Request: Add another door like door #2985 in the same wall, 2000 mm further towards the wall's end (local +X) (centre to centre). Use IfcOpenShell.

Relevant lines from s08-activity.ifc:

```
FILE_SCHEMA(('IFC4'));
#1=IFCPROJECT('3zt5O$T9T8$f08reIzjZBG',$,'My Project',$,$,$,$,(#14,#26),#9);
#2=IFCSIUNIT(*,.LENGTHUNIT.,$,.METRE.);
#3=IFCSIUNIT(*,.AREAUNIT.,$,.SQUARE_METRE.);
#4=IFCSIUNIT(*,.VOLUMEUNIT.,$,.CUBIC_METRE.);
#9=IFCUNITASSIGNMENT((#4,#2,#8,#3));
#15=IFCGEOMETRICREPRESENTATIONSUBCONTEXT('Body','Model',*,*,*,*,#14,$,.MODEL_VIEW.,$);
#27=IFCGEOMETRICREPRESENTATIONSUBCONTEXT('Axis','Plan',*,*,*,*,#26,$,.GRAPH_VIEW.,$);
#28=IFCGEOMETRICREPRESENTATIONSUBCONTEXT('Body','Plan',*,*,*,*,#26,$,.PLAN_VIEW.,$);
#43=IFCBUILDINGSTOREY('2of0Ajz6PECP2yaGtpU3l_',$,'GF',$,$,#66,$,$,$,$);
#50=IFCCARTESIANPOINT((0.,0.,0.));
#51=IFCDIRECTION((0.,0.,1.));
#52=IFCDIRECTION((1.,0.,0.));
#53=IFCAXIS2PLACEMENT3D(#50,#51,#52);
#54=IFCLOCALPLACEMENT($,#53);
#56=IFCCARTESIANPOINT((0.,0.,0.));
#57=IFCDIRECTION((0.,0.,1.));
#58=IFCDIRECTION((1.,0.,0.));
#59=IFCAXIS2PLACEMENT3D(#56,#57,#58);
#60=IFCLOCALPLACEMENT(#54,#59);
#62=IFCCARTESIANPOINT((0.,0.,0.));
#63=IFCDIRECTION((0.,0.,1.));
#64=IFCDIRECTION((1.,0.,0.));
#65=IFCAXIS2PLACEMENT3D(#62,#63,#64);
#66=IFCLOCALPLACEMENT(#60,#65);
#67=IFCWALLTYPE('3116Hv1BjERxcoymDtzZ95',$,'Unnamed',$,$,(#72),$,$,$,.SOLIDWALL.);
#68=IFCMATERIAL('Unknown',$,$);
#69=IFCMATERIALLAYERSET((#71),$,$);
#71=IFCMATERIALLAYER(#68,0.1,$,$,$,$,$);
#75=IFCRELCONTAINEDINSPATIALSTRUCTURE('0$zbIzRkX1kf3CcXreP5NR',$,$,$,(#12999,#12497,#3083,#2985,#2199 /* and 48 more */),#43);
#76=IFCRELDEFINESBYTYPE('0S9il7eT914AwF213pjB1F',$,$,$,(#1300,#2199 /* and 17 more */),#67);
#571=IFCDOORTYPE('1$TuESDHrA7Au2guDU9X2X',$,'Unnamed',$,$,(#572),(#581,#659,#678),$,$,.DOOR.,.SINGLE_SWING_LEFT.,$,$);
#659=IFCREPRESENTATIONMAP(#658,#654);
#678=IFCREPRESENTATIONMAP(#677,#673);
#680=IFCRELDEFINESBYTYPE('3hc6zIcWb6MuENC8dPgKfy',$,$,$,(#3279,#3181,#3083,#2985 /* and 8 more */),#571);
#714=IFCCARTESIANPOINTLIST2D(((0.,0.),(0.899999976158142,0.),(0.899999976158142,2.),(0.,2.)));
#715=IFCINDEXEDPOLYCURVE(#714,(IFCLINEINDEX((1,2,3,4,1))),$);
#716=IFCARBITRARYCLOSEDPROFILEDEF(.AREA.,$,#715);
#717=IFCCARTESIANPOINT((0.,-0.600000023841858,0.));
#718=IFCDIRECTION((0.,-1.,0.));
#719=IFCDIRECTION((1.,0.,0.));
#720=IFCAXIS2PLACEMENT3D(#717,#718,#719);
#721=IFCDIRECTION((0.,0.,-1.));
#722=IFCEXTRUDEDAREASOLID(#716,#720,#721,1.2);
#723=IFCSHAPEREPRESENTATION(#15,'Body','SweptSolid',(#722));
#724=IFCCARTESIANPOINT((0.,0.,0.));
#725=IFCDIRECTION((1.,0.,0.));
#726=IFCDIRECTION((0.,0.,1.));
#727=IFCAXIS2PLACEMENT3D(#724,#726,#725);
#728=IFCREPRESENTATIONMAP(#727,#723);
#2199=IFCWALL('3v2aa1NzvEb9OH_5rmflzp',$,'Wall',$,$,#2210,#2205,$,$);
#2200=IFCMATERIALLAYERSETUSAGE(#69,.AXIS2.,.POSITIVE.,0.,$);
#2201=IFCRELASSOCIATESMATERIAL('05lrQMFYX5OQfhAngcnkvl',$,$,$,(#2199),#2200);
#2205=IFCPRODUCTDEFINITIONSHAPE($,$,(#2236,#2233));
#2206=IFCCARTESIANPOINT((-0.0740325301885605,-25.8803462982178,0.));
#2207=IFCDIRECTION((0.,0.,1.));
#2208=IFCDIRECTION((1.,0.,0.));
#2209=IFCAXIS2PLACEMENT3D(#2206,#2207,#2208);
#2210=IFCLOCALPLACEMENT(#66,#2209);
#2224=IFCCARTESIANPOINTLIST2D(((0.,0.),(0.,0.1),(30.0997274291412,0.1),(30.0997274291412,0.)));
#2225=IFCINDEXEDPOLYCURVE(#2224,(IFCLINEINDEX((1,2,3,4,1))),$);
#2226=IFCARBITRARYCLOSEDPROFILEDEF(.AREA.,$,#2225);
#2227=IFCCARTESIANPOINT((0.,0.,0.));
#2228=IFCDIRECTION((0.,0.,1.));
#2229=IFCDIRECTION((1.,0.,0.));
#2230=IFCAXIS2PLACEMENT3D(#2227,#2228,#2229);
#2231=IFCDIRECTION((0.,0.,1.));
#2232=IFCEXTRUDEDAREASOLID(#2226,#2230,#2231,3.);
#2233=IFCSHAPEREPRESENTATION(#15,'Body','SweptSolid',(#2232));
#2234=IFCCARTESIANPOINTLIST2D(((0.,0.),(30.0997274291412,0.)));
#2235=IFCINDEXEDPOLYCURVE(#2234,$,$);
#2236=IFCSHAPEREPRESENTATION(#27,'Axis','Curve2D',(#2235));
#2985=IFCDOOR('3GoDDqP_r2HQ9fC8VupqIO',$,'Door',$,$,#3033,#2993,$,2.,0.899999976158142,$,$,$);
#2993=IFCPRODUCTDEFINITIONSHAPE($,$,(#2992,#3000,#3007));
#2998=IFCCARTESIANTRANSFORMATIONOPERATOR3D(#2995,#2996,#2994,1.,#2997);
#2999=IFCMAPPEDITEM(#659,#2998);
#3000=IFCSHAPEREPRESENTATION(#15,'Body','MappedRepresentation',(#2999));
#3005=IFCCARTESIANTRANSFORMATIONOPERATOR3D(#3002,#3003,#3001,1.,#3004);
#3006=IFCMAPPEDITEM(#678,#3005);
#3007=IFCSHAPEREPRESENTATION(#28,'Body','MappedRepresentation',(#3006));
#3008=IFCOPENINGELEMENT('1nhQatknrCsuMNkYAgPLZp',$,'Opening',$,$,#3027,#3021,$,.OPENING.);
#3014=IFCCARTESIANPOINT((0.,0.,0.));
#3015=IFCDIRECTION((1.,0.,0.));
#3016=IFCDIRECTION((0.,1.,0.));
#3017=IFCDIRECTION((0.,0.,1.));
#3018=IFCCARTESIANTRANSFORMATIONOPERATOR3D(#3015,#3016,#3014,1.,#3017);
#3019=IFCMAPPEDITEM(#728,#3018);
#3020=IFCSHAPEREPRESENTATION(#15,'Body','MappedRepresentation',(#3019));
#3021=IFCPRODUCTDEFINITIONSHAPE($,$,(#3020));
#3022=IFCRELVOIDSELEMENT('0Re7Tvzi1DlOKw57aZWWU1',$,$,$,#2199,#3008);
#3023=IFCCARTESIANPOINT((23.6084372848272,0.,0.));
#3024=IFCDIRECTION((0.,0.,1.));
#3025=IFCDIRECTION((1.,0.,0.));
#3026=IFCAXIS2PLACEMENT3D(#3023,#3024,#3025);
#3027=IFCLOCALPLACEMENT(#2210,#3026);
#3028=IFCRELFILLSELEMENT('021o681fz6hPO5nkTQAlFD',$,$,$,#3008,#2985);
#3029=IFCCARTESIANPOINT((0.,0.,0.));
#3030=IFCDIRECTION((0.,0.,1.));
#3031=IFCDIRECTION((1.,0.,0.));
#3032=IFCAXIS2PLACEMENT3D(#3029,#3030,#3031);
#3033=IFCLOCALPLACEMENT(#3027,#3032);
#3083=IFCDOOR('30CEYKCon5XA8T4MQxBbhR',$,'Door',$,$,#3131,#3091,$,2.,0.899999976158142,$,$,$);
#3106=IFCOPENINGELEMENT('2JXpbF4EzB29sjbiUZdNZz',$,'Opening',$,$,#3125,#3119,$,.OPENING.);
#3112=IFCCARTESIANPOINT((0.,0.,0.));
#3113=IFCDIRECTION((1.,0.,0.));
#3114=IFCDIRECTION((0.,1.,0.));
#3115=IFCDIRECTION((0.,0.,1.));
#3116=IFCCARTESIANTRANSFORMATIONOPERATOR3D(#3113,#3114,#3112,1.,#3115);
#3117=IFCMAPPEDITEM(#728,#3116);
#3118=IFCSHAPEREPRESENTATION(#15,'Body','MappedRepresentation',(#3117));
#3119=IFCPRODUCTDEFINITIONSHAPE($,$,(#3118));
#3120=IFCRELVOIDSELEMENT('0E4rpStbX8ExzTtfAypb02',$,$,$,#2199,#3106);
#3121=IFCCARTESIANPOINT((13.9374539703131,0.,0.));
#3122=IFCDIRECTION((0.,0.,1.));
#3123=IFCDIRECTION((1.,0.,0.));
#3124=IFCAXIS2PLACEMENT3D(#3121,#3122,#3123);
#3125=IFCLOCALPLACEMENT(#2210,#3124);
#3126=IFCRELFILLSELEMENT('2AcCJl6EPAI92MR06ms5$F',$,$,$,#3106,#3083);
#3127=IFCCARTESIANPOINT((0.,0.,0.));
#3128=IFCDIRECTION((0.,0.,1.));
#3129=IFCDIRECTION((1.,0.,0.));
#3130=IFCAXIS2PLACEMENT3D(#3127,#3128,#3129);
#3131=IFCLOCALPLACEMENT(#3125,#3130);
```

```python
import ifcopenshell
import ifcopenshell.api.feature
import ifcopenshell.api.geometry
import ifcopenshell.api.root
import ifcopenshell.geom
import ifcopenshell.util.element
import ifcopenshell.util.placement
import ifcopenshell.util.shape
import ifcopenshell.util.unit

model = ifcopenshell.open("s08-activity.ifc")
unit_scale = ifcopenshell.util.unit.calculate_unit_scale(model)
settings = ifcopenshell.geom.settings()


def volume(element):
    """Net volume in cubic metres, openings subtracted."""
    shape = ifcopenshell.geom.create_shape(settings, element)
    return ifcopenshell.util.shape.get_volume(shape.geometry)


door = model.by_guid("3GoDDqP_r2HQ9fC8VupqIO")
opening = door.FillsVoids[0].RelatingOpeningElement
wall = opening.VoidsElements[0].RelatingBuildingElement
before = volume(wall)
shift = ifcopenshell.util.placement.get_local_placement(wall.ObjectPlacement)[:3, 0] * 2 / unit_scale

# copy_class copies the void relationship, type, container and properties, but no geometry.
new_opening = ifcopenshell.api.root.copy_class(model, product=opening)
new_opening.Representation = ifcopenshell.util.element.copy_deep(
    model, opening.Representation, exclude=["IfcGeometricRepresentationContext", "IfcRepresentationMap"]
)
new_door = ifcopenshell.api.root.copy_class(model, product=door)
new_door.Representation = ifcopenshell.util.element.copy_deep(
    model, door.Representation, exclude=["IfcGeometricRepresentationContext", "IfcRepresentationMap"]
)
ifcopenshell.api.feature.add_filling(model, opening=new_opening, element=new_door)

for old, new in ((opening, new_opening), (door, new_door)):
    matrix = ifcopenshell.util.placement.get_local_placement(old.ObjectPlacement)
    matrix[:3, 3] += shift
    ifcopenshell.api.geometry.edit_object_placement(model, product=new, matrix=matrix, is_si=False)

after = volume(wall)

print(f"wall volume {before:.3f} -> {after:.3f} m3")

model.write("s08-activity_edited.ifc")
```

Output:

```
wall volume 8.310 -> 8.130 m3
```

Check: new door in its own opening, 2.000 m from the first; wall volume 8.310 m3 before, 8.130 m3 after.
